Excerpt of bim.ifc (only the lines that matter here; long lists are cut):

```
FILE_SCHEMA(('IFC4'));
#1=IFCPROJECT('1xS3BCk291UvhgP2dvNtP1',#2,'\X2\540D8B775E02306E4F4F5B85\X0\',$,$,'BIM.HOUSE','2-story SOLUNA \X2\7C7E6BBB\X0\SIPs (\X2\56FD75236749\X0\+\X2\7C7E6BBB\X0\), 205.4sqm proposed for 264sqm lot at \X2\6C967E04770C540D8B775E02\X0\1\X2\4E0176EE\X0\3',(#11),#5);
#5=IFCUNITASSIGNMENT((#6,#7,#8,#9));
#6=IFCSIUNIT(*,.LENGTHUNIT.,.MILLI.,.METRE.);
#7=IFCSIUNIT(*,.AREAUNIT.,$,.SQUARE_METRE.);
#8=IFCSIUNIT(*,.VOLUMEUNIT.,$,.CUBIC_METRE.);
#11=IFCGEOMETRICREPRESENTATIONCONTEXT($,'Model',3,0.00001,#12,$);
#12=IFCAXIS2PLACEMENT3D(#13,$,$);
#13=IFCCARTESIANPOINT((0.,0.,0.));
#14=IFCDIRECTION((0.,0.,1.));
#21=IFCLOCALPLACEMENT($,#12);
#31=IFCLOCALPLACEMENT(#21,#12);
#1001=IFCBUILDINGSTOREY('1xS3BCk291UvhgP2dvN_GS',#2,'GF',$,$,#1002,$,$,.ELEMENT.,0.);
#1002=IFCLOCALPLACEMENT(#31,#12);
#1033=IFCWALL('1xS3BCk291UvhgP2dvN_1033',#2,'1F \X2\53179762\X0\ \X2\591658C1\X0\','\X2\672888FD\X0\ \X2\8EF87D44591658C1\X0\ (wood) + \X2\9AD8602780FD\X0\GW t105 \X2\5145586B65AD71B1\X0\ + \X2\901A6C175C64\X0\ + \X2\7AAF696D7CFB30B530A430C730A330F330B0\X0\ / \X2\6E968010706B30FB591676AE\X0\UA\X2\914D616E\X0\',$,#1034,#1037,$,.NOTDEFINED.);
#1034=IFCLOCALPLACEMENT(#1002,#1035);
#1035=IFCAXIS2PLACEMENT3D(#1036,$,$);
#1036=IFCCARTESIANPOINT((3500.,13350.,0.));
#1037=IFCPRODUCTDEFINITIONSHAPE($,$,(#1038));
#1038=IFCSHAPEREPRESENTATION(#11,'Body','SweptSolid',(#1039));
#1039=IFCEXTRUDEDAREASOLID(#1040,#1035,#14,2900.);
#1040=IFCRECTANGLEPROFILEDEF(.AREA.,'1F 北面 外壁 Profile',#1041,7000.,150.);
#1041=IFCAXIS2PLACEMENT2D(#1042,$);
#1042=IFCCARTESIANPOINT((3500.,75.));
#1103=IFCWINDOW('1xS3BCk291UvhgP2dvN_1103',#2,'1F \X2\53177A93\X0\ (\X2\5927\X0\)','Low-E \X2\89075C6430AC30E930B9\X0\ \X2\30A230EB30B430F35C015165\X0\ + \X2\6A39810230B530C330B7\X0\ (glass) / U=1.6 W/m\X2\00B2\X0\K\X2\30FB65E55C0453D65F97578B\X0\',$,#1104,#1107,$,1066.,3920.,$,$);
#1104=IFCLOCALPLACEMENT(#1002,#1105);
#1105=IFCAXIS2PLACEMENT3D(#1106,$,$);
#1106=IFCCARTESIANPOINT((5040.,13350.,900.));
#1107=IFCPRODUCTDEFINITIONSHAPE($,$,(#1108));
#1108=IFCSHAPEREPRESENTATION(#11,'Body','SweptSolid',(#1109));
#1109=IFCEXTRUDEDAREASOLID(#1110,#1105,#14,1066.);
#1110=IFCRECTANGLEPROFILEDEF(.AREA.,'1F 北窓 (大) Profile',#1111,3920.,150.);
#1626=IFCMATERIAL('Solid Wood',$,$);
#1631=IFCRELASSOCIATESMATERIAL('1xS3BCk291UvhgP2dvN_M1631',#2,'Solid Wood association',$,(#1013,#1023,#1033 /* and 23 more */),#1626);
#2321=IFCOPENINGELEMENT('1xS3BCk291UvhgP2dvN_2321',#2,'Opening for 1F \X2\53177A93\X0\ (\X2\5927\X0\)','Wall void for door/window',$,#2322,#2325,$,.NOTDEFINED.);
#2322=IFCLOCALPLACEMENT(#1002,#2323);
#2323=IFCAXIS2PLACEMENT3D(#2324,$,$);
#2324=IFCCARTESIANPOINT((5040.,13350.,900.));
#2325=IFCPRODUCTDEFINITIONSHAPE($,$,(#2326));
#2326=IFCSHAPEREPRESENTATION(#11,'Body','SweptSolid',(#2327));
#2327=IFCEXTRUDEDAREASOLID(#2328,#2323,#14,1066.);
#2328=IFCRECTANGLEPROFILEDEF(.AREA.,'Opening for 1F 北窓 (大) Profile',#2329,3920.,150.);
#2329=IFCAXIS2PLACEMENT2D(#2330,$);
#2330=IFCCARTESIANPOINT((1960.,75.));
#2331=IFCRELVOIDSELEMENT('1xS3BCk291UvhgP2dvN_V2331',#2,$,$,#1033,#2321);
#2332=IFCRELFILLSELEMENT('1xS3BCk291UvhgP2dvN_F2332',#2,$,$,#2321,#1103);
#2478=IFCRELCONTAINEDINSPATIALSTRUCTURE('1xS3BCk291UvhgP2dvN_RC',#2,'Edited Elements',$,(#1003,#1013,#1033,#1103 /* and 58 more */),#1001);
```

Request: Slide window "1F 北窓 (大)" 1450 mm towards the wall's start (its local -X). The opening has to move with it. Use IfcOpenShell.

```python
import ifcopenshell
import ifcopenshell.api.geometry
import ifcopenshell.util.placement
import ifcopenshell.util.unit

model = ifcopenshell.open("bim.ifc")
unit_scale = ifcopenshell.util.unit.calculate_unit_scale(model)

window = model.by_guid("1xS3BCk291UvhgP2dvN_1103")
opening = window.FillsVoids[0].RelatingOpeningElement
wall = opening.VoidsElements[0].RelatingBuildingElement

wall_matrix = ifcopenshell.util.placement.get_local_placement(wall.ObjectPlacement)
shift = wall_matrix[:3, 0] * -1.45 / unit_scale
before = ifcopenshell.util.placement.get_local_placement(window.ObjectPlacement)[:3, 3].copy()

# The window is not placed relative to its opening, so move both.
for product in (opening, window):
    matrix = ifcopenshell.util.placement.get_local_placement(product.ObjectPlacement)
    matrix[:3, 3] += shift
    ifcopenshell.api.geometry.edit_object_placement(model, product=product, matrix=matrix, is_si=False)

after = ifcopenshell.util.placement.get_local_placement(window.ObjectPlacement)[:3, 3]
print("window moved by", (after - before).round(3) + 0.0)

model.write("bim_v2.ifc")
```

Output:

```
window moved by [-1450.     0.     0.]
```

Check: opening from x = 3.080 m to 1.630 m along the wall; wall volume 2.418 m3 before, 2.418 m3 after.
